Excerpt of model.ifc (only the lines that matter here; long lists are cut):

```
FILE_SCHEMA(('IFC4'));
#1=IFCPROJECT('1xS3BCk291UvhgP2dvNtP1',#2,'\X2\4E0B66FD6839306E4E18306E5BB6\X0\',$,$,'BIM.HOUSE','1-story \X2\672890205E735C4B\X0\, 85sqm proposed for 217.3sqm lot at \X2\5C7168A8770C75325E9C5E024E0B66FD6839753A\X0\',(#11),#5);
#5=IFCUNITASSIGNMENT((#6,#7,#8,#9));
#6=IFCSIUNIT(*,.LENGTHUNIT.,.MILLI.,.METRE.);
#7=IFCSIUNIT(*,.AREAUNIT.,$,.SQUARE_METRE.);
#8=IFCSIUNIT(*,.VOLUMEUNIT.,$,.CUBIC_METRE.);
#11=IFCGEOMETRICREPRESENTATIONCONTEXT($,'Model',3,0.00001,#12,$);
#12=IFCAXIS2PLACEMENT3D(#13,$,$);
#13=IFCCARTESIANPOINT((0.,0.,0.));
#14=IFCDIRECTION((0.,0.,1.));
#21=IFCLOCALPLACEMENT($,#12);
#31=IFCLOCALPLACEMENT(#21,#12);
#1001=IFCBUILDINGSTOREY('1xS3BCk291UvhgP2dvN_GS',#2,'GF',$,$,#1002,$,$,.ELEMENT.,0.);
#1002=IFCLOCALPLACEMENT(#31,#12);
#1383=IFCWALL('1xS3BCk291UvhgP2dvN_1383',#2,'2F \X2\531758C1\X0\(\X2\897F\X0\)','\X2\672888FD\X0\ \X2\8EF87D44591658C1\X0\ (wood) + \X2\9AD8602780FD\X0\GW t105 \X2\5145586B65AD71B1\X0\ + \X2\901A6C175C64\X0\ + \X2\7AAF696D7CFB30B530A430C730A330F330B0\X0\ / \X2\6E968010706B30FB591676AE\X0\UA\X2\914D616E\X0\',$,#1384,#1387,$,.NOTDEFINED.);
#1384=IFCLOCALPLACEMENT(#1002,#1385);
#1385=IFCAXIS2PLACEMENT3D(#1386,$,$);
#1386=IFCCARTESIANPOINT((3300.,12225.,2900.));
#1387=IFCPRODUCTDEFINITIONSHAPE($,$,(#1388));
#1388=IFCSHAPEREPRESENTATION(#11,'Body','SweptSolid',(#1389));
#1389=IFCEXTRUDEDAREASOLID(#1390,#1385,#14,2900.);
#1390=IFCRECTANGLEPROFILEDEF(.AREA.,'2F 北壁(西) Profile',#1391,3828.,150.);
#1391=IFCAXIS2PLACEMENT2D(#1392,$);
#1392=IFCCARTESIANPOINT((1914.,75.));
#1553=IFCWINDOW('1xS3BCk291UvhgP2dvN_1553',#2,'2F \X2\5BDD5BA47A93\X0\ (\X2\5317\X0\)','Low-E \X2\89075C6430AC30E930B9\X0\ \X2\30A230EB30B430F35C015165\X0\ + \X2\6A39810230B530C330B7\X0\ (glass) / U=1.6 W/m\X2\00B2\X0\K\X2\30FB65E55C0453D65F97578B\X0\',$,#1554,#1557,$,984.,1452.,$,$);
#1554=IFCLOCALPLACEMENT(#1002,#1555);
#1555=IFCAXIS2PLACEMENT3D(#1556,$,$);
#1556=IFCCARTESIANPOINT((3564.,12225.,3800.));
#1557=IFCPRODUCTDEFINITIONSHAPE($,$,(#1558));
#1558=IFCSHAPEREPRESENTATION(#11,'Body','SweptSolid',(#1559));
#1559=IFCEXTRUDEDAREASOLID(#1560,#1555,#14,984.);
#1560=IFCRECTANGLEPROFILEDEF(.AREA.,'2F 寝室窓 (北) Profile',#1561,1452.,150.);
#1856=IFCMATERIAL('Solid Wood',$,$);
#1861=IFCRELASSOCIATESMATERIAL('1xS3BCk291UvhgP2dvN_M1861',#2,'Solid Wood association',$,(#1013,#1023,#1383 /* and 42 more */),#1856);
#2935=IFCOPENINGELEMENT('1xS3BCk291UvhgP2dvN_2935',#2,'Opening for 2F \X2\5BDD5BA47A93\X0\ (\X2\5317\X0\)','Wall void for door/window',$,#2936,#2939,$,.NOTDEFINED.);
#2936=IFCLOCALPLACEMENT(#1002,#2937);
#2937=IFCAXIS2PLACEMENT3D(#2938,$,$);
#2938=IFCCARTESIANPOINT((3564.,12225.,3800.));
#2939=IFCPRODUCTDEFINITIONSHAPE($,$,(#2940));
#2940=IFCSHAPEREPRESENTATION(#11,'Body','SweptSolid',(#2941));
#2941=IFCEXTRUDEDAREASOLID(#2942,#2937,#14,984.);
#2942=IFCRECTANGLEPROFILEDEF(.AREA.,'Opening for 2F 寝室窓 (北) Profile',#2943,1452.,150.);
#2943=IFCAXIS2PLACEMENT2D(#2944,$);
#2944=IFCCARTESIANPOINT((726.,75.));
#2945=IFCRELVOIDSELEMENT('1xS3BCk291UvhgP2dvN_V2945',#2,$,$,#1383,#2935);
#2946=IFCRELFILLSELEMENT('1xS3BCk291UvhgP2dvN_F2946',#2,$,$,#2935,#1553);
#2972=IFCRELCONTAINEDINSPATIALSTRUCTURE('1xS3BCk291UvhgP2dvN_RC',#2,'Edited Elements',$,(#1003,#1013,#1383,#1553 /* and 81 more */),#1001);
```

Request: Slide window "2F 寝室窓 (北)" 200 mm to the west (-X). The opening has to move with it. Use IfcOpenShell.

```python
import ifcopenshell
import ifcopenshell.api.geometry
import ifcopenshell.util.placement
import ifcopenshell.util.unit

model = ifcopenshell.open("model.ifc")
unit_scale = ifcopenshell.util.unit.calculate_unit_scale(model)

window = model.by_guid("1xS3BCk291UvhgP2dvN_1553")
opening = window.FillsVoids[0].RelatingOpeningElement
wall = opening.VoidsElements[0].RelatingBuildingElement

wall_matrix = ifcopenshell.util.placement.get_local_placement(wall.ObjectPlacement)
shift = wall_matrix[:3, 0] * -0.2 / unit_scale
before = ifcopenshell.util.placement.get_local_placement(window.ObjectPlacement)[:3, 3].copy()

# The window is not placed relative to its opening, so move both.
for product in (opening, window):
    matrix = ifcopenshell.util.placement.get_local_placement(product.ObjectPlacement)
    matrix[:3, 3] += shift
    ifcopenshell.api.geometry.edit_object_placement(model, product=product, matrix=matrix, is_si=False)

after = ifcopenshell.util.placement.get_local_placement(window.ObjectPlacement)[:3, 3]
print("window moved by", (after - before).round(3) + 0.0)

model.write("model_edited.ifc")
```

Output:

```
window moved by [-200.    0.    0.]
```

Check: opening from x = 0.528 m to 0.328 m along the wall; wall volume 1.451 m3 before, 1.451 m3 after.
